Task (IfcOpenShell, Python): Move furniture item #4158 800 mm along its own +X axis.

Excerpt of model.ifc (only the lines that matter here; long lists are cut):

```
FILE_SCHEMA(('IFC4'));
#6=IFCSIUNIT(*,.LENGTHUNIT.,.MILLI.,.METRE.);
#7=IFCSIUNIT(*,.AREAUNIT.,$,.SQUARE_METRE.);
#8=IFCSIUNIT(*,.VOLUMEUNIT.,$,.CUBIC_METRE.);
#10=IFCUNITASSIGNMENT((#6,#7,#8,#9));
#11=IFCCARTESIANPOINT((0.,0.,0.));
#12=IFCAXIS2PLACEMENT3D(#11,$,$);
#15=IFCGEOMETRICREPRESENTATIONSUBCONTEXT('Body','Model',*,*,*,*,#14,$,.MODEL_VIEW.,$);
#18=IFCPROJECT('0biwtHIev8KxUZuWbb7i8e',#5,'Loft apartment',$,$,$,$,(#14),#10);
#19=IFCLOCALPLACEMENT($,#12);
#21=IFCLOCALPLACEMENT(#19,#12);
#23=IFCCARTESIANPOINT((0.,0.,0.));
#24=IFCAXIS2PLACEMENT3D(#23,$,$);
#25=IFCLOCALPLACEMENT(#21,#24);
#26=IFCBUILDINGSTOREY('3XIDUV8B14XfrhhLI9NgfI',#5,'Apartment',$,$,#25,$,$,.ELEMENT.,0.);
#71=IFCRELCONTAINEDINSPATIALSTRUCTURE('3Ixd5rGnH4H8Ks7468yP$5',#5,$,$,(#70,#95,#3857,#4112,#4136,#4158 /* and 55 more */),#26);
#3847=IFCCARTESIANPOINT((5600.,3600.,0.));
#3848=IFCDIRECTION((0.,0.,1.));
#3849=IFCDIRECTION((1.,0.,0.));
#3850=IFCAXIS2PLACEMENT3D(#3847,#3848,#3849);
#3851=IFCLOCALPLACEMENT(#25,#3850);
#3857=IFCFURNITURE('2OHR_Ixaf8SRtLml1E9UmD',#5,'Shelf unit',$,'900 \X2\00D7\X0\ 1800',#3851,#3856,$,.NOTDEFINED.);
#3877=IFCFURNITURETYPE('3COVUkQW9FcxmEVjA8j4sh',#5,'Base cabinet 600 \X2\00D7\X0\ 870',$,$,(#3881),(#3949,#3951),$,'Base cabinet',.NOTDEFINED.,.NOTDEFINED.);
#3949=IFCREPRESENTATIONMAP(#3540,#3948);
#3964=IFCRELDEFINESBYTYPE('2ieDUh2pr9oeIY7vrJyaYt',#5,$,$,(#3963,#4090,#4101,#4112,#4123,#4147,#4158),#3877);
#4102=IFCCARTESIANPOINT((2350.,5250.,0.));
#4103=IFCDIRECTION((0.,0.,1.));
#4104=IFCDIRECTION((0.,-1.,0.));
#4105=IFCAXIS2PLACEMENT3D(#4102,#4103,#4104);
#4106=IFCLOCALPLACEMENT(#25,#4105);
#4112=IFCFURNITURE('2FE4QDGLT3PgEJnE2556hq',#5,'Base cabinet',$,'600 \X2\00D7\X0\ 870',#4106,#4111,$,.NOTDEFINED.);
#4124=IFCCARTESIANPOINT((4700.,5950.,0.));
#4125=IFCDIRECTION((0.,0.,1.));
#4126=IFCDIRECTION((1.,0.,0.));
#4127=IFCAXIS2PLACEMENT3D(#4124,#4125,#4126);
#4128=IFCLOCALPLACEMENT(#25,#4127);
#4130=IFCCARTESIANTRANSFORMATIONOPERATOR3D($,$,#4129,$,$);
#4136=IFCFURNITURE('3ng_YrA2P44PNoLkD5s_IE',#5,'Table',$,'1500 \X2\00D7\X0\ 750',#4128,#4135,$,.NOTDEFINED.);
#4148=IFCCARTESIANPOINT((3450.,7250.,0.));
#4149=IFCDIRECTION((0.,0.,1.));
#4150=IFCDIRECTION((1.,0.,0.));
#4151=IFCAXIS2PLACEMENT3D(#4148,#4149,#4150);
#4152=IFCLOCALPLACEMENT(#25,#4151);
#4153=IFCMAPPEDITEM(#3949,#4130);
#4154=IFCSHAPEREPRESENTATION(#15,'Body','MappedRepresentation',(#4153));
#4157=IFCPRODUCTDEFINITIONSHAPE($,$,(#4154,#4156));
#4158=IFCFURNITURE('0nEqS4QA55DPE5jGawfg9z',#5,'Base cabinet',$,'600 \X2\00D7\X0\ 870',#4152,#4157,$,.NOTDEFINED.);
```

```python
import ifcopenshell
import ifcopenshell.api.geometry
import ifcopenshell.util.placement
import ifcopenshell.util.unit

model = ifcopenshell.open("model.ifc")
unit_scale = ifcopenshell.util.unit.calculate_unit_scale(model)

item = model.by_guid("0nEqS4QA55DPE5jGawfg9z")
matrix = ifcopenshell.util.placement.get_local_placement(item.ObjectPlacement)
matrix[:3, 3] += matrix[:3, 0] * 0.8 / unit_scale
ifcopenshell.api.geometry.edit_object_placement(model, product=item, matrix=matrix, is_si=False)

print(ifcopenshell.util.placement.get_local_placement(item.ObjectPlacement).round(3) + 0.0)

model.write("model_v2.ifc")
```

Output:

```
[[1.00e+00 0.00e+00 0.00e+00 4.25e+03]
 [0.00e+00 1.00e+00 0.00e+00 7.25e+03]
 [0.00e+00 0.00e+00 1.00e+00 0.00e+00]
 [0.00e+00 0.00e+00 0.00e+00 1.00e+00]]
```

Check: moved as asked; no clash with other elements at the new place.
